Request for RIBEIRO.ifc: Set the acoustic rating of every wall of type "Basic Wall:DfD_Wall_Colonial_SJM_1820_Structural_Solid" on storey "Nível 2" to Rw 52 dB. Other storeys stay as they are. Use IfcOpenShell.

First a look at what the model holds.

```python
import ifcopenshell
import ifcopenshell.util.element

model = ifcopenshell.open("RIBEIRO.ifc")
print(model.schema)
storey = next(s for s in model.by_type("IfcBuildingStorey") if s.Name == "Nível 2")
walls = [e for e in ifcopenshell.util.element.get_decomposition(storey) if e.is_a("IfcWall")]
seen = {}
for e in walls:
    element_type = ifcopenshell.util.element.get_type(e)
    key = (element_type.Name if element_type != e and element_type else None, ifcopenshell.util.element.get_pset(e, "Pset_WallCommon", "AcousticRating"))
    seen[key] = seen.get(key, 0) + 1
for (name, value), count in sorted(seen.items(), key=str):
    print(count, "x", name, "|", value)
```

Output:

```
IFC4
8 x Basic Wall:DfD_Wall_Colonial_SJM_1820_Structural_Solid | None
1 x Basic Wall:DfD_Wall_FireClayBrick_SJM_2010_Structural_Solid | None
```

```python
import ifcopenshell
import ifcopenshell.api.pset
import ifcopenshell.util.element

model = ifcopenshell.open("RIBEIRO.ifc")

storey = next(s for s in model.by_type("IfcBuildingStorey") if s.Name == "Nível 2")
walls = [e for e in ifcopenshell.util.element.get_decomposition(storey) if e.is_a("IfcWall")]

count = 0
for e in walls:
    element_type = ifcopenshell.util.element.get_type(e)
    if element_type in (None, e) or element_type.Name != "Basic Wall:DfD_Wall_Colonial_SJM_1820_Structural_Solid":
        continue
    # add_pset returns the element's existing set when there is one.
    pset = ifcopenshell.api.pset.add_pset(model, product=e, name="Pset_WallCommon")
    ifcopenshell.api.pset.edit_pset(model, pset=pset, properties={"AcousticRating": "Rw 52 dB"})
    count += 1

print(count, "walls updated")

model.write("RIBEIRO_edited.ifc")
```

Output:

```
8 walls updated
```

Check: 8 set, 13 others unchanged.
